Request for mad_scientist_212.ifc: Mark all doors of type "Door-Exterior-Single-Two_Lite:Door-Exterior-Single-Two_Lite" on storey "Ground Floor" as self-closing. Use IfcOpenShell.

First a look at what the model holds.

```python
import ifcopenshell
import ifcopenshell.util.element

model = ifcopenshell.open("mad_scientist_212.ifc")
print(model.schema)
storey = next(s for s in model.by_type("IfcBuildingStorey") if s.Name == "Ground Floor")
doors = [e for e in ifcopenshell.util.element.get_decomposition(storey) if e.is_a("IfcDoor")]
seen = {}
for e in doors:
    element_type = ifcopenshell.util.element.get_type(e)
    key = (element_type.Name if element_type != e and element_type else None, ifcopenshell.util.element.get_pset(e, "Pset_DoorCommon", "SelfClosing"))
    seen[key] = seen.get(key, 0) + 1
for (name, value), count in sorted(seen.items(), key=str):
    print(count, "x", name, "|", value)
```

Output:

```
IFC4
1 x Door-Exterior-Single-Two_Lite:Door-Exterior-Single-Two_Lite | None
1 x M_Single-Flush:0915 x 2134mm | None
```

```python
import ifcopenshell
import ifcopenshell.api.pset
import ifcopenshell.util.element

model = ifcopenshell.open("mad_scientist_212.ifc")

storey = next(s for s in model.by_type("IfcBuildingStorey") if s.Name == "Ground Floor")
doors = [e for e in ifcopenshell.util.element.get_decomposition(storey) if e.is_a("IfcDoor")]

count = 0
for e in doors:
    element_type = ifcopenshell.util.element.get_type(e)
    if element_type in (None, e) or element_type.Name != "Door-Exterior-Single-Two_Lite:Door-Exterior-Single-Two_Lite":
        continue
    # add_pset returns the element's existing set when there is one.
    pset = ifcopenshell.api.pset.add_pset(model, product=e, name="Pset_DoorCommon")
    ifcopenshell.api.pset.edit_pset(model, pset=pset, properties={"SelfClosing": True})
    count += 1

print(count, "doors updated")

model.write("mad_scientist_212_v2.ifc")
```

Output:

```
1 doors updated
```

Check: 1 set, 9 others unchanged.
